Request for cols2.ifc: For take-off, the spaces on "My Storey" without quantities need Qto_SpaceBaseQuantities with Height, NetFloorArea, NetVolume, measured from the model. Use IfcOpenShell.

First a look at what the model holds.

```python
import ifcopenshell
import ifcopenshell.util.element
import ifcopenshell.util.unit

model = ifcopenshell.open("cols2.ifc")
print(model.schema)
for unit_type in ("LENGTHUNIT", "AREAUNIT", "VOLUMEUNIT"):
    print(unit_type, ifcopenshell.util.unit.calculate_unit_scale(model, unit_type))
storey = next(s for s in model.by_type("IfcBuildingStorey") if s.Name == "My Storey")
spaces = [e for e in ifcopenshell.util.element.get_decomposition(storey) if e.is_a("IfcSpace")]
for e in sorted(spaces, key=lambda e: e.id()):
    print(e.id(), e.is_a(), e.Name, list(ifcopenshell.util.element.get_psets(e, qtos_only=True)), sep=" | ")
```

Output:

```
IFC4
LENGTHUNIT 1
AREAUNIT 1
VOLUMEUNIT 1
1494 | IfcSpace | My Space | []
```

```python
import ifcopenshell
import ifcopenshell.api.pset
import ifcopenshell.geom
import ifcopenshell.util.element
import ifcopenshell.util.shape
import ifcopenshell.util.unit

model = ifcopenshell.open("cols2.ifc")
unit_scale = ifcopenshell.util.unit.calculate_unit_scale(model)
area_scale = ifcopenshell.util.unit.calculate_unit_scale(model, "AREAUNIT")
volume_scale = ifcopenshell.util.unit.calculate_unit_scale(model, "VOLUMEUNIT")
settings = ifcopenshell.geom.settings()

storey = next(s for s in model.by_type("IfcBuildingStorey") if s.Name == "My Storey")
spaces = [e for e in ifcopenshell.util.element.get_decomposition(storey) if e.is_a("IfcSpace")]

for e in sorted(spaces, key=lambda e: e.id()):
    if ifcopenshell.util.element.get_psets(e, qtos_only=True, should_inherit=False):
        continue
    # Geometry comes back in metres, in the element's own axes.
    shape = ifcopenshell.geom.create_shape(settings, e)
    values = {
        "Height": ifcopenshell.util.shape.get_z(shape.geometry) / unit_scale,
        "NetFloorArea": ifcopenshell.util.shape.get_footprint_area(shape.geometry) / area_scale,
        "NetVolume": ifcopenshell.util.shape.get_volume(shape.geometry) / volume_scale,
    }
    qto = ifcopenshell.api.pset.add_qto(model, product=e, name="Qto_SpaceBaseQuantities")
    ifcopenshell.api.pset.edit_qto(model, qto=qto, properties=values)
    print(e.id(), {k: round(v, 3) for k, v in values.items()})

model.write("cols2_v2.ifc")
```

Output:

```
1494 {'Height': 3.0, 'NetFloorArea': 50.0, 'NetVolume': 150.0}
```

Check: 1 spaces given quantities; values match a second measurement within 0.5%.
